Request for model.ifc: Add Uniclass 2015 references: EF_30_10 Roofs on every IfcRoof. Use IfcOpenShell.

First a look at what the model holds.

```python
import ifcopenshell

model = ifcopenshell.open("model.ifc")
print(model.schema)
print("classifications:", [c.Name for c in model.by_type("IfcClassification")])
for ifc_class in ("IfcDoor", "IfcRoof", "IfcStair", "IfcWall", "IfcWindow"):
    print(ifc_class, len(model.by_type(ifc_class)))
```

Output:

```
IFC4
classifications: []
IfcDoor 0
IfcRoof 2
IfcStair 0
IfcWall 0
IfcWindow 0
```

```python
import ifcopenshell
import ifcopenshell.api.classification

model = ifcopenshell.open("model.ifc")

system = ifcopenshell.api.classification.add_classification(model, classification="Uniclass 2015")

codes = {
    "IfcRoof": ("EF_30_10", "Roofs"),
}
for ifc_class, (code, name) in codes.items():
    products = model.by_type(ifc_class)
    ifcopenshell.api.classification.add_reference(
        model, products=products, classification=system, identification=code, name=name
    )
    print(code, len(products))

model.write("model_updated.ifc")
```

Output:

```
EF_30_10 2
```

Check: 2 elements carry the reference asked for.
